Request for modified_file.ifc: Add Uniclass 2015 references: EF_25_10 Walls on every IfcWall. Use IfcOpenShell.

First a look at what the model holds.

```python
import ifcopenshell

model = ifcopenshell.open("modified_file.ifc")
print(model.schema)
print("classifications:", [c.Name for c in model.by_type("IfcClassification")])
for ifc_class in ("IfcDoor", "IfcRoof", "IfcStair", "IfcWall", "IfcWindow"):
    print(ifc_class, len(model.by_type(ifc_class)))
```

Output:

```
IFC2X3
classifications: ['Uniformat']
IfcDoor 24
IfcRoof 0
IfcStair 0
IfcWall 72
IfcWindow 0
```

```python
import ifcopenshell
import ifcopenshell.api.classification

model = ifcopenshell.open("modified_file.ifc")

# IFC2X3 requires Source and Edition and has no link from the project to the system.
system = model.create_entity("IfcClassification", Source="NBS", Edition="2015", Name="Uniclass 2015")

codes = {
    "IfcWall": ("EF_25_10", "Walls"),
}
for ifc_class, (code, name) in codes.items():
    products = model.by_type(ifc_class)
    ifcopenshell.api.classification.add_reference(
        model, products=products, classification=system, identification=code, name=name
    )
    print(code, len(products))

model.write("modified_file_edited.ifc")
```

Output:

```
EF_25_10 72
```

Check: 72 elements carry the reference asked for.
